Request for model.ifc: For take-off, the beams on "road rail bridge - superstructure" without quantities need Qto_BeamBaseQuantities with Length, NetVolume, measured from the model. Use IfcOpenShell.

First a look at what the model holds.

```python
import ifcopenshell
import ifcopenshell.util.element
import ifcopenshell.util.unit

model = ifcopenshell.open("model.ifc")
print(model.schema)
for unit_type in ("LENGTHUNIT", "AREAUNIT", "VOLUMEUNIT"):
    print(unit_type, ifcopenshell.util.unit.calculate_unit_scale(model, unit_type))
storey = next(s for s in model.by_type("IfcBuildingStorey") if s.Name == "road rail bridge - superstructure")
beams = [e for e in ifcopenshell.util.element.get_decomposition(storey) if e.is_a("IfcBeam")]
for e in sorted(beams, key=lambda e: e.id()):
    print(e.id(), e.is_a(), e.Name, list(ifcopenshell.util.element.get_psets(e, qtos_only=True)), sep=" | ")
```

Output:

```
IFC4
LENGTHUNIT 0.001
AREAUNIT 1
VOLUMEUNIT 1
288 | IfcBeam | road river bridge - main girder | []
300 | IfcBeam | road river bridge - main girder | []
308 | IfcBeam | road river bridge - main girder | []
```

```python
import ifcopenshell
import ifcopenshell.api.pset
import ifcopenshell.geom
import ifcopenshell.util.element
import ifcopenshell.util.shape
import ifcopenshell.util.unit

model = ifcopenshell.open("model.ifc")
unit_scale = ifcopenshell.util.unit.calculate_unit_scale(model)
volume_scale = ifcopenshell.util.unit.calculate_unit_scale(model, "VOLUMEUNIT")
settings = ifcopenshell.geom.settings()

storey = next(s for s in model.by_type("IfcBuildingStorey") if s.Name == "road rail bridge - superstructure")
beams = [e for e in ifcopenshell.util.element.get_decomposition(storey) if e.is_a("IfcBeam")]

for e in sorted(beams, key=lambda e: e.id()):
    if ifcopenshell.util.element.get_psets(e, qtos_only=True, should_inherit=False):
        continue
    # Geometry comes back in metres, in the element's own axes.
    shape = ifcopenshell.geom.create_shape(settings, e)
    values = {
        "Length": ifcopenshell.util.shape.get_max_xyz(shape.geometry) / unit_scale,
        "NetVolume": ifcopenshell.util.shape.get_volume(shape.geometry) / volume_scale,
    }
    qto = ifcopenshell.api.pset.add_qto(model, product=e, name="Qto_BeamBaseQuantities")
    ifcopenshell.api.pset.edit_qto(model, qto=qto, properties=values)
    print(e.id(), {k: round(v, 3) for k, v in values.items()})

model.write("model_rev.ifc")
```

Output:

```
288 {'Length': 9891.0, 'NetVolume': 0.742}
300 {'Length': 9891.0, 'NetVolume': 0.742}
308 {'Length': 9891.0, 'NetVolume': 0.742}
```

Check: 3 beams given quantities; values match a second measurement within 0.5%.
